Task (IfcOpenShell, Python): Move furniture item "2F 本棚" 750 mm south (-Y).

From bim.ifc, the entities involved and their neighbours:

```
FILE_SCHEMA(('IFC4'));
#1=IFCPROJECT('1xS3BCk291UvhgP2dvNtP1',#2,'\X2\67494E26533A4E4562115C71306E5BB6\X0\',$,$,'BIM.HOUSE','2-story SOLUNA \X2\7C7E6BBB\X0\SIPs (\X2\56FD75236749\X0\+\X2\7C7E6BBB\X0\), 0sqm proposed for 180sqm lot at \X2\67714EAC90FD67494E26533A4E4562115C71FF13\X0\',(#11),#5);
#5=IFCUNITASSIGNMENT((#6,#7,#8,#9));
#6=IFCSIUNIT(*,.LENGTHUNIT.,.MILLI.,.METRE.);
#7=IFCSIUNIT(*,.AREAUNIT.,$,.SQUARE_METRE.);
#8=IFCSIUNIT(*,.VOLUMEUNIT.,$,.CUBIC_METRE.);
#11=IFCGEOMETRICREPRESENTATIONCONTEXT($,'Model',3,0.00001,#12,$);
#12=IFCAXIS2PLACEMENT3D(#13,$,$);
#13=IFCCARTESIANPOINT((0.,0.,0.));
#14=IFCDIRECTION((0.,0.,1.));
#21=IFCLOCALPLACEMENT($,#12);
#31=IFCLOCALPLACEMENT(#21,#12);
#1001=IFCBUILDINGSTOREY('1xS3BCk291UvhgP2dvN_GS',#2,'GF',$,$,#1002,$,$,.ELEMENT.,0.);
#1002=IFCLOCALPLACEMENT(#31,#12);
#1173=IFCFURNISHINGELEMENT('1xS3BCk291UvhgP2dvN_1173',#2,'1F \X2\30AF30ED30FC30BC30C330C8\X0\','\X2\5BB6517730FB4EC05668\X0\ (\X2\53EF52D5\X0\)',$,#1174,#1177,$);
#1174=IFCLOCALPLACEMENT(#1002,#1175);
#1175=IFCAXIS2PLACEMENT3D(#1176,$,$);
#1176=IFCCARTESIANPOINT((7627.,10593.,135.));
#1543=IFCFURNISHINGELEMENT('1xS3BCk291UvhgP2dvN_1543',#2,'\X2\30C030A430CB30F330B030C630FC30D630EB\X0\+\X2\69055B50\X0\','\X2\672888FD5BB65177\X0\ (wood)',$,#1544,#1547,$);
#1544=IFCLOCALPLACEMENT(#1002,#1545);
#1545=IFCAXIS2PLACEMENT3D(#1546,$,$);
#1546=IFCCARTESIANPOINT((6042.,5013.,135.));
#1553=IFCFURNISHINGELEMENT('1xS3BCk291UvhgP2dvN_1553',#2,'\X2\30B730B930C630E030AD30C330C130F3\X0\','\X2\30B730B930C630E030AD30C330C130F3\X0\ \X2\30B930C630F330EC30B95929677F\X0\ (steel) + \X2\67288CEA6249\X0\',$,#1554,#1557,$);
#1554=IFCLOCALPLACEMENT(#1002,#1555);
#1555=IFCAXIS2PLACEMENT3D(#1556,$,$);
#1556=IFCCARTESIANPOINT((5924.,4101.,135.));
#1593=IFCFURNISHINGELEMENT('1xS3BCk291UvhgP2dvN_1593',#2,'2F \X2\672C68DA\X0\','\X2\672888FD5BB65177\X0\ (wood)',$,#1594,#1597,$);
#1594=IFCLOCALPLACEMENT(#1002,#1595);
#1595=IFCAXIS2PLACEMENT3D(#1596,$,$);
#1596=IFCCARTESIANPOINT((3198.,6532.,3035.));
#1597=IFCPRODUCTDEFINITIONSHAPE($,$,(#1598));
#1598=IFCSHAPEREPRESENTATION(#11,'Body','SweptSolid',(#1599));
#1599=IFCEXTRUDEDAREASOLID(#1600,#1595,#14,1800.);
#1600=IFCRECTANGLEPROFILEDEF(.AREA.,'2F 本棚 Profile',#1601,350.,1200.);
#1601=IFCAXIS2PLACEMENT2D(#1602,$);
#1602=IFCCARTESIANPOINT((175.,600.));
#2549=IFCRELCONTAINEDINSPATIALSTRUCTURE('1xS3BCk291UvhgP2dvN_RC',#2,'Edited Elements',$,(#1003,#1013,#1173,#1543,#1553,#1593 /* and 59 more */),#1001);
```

```python
import ifcopenshell
import ifcopenshell.api.geometry
import ifcopenshell.util.placement
import ifcopenshell.util.unit

model = ifcopenshell.open("bim.ifc")
unit_scale = ifcopenshell.util.unit.calculate_unit_scale(model)

item = model.by_id(1593)
matrix = ifcopenshell.util.placement.get_local_placement(item.ObjectPlacement)
matrix[1, 3] -= 0.75 / unit_scale
ifcopenshell.api.geometry.edit_object_placement(model, product=item, matrix=matrix, is_si=False)

print(ifcopenshell.util.placement.get_local_placement(item.ObjectPlacement).round(3) + 0.0)

model.write("bim_v2.ifc")
```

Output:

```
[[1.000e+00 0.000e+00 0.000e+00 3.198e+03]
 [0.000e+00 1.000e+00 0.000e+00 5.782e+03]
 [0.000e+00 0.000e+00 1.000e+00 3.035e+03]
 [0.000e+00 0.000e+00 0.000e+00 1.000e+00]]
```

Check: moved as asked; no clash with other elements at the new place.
